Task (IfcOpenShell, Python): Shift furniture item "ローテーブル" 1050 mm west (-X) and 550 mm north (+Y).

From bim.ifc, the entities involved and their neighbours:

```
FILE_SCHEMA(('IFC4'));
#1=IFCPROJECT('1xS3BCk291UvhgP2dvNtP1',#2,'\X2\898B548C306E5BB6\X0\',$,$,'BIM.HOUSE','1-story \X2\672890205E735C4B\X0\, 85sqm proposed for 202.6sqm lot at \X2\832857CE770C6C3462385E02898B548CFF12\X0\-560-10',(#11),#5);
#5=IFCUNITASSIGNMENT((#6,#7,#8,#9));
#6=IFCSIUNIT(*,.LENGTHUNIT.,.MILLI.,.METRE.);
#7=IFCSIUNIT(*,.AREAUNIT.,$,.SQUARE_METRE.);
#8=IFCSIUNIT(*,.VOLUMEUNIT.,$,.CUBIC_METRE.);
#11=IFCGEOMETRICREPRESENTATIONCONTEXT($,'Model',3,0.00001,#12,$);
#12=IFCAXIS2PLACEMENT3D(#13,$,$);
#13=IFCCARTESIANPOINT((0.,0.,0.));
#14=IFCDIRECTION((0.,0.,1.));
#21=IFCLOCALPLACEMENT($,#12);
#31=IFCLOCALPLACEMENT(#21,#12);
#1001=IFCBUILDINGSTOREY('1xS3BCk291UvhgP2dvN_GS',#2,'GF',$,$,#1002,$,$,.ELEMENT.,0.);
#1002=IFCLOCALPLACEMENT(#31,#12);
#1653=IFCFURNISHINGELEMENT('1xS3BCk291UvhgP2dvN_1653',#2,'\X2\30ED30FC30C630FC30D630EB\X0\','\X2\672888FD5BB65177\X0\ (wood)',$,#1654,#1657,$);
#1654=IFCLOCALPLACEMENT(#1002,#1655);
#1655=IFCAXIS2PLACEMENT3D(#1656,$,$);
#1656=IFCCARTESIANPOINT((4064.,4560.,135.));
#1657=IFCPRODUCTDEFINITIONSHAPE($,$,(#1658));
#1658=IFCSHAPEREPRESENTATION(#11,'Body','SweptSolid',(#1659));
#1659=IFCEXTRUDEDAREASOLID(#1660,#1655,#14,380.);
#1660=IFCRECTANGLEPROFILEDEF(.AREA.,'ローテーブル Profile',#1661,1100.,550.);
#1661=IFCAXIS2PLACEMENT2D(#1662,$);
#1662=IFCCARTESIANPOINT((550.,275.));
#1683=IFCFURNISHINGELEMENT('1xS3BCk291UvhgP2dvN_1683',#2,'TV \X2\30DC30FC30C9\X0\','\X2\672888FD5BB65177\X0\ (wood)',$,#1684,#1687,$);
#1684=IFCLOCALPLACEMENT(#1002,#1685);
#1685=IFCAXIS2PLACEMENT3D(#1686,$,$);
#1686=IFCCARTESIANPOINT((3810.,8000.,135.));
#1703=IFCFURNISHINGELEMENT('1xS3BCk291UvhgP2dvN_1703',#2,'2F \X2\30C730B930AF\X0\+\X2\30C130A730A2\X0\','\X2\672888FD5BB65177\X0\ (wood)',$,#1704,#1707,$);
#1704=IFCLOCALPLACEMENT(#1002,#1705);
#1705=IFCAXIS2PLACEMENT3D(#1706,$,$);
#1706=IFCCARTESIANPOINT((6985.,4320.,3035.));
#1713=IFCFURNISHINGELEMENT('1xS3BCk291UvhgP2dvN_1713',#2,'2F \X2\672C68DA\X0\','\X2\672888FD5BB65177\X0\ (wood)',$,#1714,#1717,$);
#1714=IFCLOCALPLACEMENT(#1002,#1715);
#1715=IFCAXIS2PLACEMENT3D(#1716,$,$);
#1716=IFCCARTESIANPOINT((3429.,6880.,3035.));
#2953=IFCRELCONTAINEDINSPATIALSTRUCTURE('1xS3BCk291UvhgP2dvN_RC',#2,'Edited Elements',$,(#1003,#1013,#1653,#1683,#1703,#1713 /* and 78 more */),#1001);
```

```python
import ifcopenshell
import ifcopenshell.api.geometry
import ifcopenshell.util.placement
import ifcopenshell.util.unit

model = ifcopenshell.open("bim.ifc")
unit_scale = ifcopenshell.util.unit.calculate_unit_scale(model)

item = model.by_id(1653)
matrix = ifcopenshell.util.placement.get_local_placement(item.ObjectPlacement)
matrix[0, 3] -= 1.05 / unit_scale
matrix[1, 3] += 0.55 / unit_scale
ifcopenshell.api.geometry.edit_object_placement(model, product=item, matrix=matrix, is_si=False)

print(ifcopenshell.util.placement.get_local_placement(item.ObjectPlacement).round(3) + 0.0)

model.write("bim-out.ifc")
```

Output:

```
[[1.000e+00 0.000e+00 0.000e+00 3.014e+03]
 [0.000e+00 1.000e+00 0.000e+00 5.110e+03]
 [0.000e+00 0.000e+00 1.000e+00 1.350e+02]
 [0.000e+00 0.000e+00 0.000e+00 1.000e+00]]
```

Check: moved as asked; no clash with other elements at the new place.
